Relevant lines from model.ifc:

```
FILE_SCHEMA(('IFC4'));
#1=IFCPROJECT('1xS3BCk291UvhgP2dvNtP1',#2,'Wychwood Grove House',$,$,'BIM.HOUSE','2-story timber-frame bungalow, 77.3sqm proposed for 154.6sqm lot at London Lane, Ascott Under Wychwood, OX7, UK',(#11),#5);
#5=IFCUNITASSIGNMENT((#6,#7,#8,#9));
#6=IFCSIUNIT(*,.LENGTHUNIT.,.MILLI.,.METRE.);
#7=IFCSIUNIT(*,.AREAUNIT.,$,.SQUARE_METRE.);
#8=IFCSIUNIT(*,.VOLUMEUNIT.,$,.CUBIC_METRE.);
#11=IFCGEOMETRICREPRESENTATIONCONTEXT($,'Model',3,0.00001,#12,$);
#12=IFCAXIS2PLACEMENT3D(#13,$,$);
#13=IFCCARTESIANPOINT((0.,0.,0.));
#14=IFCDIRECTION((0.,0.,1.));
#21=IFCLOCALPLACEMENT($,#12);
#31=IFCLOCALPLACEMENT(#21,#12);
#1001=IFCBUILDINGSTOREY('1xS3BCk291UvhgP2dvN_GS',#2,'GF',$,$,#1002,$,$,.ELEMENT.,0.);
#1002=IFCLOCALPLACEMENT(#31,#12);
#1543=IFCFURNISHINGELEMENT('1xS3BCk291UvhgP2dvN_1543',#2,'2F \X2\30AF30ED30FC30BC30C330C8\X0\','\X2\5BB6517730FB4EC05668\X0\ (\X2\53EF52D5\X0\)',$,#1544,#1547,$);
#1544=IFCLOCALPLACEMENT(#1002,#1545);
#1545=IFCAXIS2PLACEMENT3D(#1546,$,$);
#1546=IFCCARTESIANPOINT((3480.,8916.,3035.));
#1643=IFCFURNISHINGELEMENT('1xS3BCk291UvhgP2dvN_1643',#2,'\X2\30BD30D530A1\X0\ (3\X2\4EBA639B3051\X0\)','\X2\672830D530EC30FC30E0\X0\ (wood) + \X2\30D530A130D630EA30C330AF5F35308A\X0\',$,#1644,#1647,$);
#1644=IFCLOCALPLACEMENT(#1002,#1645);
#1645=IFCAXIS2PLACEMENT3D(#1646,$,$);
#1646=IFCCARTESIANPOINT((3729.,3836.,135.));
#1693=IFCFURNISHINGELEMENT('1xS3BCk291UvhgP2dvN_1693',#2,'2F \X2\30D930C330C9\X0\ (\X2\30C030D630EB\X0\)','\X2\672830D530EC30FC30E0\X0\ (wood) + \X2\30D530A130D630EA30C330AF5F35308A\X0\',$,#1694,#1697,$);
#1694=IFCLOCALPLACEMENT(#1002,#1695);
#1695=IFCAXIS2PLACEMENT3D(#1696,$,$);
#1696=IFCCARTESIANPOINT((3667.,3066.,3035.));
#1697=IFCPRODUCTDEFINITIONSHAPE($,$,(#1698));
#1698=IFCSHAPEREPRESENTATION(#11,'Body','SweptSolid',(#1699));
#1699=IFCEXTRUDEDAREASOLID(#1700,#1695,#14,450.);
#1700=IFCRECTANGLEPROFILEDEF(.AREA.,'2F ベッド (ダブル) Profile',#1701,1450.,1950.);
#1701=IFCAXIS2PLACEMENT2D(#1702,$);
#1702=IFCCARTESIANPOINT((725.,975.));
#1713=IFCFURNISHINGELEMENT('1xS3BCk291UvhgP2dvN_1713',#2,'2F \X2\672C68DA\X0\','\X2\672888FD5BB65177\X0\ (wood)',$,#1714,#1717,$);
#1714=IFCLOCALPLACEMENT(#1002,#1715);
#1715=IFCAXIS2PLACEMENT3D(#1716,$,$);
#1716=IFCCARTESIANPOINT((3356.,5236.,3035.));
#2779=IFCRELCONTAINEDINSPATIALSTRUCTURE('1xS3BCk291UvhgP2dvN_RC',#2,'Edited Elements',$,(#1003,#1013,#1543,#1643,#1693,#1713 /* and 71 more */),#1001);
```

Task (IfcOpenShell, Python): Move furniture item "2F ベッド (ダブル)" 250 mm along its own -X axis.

```python
import ifcopenshell
import ifcopenshell.api.geometry
import ifcopenshell.util.placement
import ifcopenshell.util.unit

model = ifcopenshell.open("model.ifc")
unit_scale = ifcopenshell.util.unit.calculate_unit_scale(model)

item = model.by_id(1693)
matrix = ifcopenshell.util.placement.get_local_placement(item.ObjectPlacement)
matrix[:3, 3] -= matrix[:3, 0] * 0.25 / unit_scale
ifcopenshell.api.geometry.edit_object_placement(model, product=item, matrix=matrix, is_si=False)

print(ifcopenshell.util.placement.get_local_placement(item.ObjectPlacement).round(3) + 0.0)

model.write("model_edited.ifc")
```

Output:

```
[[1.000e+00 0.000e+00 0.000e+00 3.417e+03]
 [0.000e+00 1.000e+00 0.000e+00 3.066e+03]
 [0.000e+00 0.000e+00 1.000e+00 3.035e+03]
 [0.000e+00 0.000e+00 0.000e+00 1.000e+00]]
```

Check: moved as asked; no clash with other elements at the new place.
